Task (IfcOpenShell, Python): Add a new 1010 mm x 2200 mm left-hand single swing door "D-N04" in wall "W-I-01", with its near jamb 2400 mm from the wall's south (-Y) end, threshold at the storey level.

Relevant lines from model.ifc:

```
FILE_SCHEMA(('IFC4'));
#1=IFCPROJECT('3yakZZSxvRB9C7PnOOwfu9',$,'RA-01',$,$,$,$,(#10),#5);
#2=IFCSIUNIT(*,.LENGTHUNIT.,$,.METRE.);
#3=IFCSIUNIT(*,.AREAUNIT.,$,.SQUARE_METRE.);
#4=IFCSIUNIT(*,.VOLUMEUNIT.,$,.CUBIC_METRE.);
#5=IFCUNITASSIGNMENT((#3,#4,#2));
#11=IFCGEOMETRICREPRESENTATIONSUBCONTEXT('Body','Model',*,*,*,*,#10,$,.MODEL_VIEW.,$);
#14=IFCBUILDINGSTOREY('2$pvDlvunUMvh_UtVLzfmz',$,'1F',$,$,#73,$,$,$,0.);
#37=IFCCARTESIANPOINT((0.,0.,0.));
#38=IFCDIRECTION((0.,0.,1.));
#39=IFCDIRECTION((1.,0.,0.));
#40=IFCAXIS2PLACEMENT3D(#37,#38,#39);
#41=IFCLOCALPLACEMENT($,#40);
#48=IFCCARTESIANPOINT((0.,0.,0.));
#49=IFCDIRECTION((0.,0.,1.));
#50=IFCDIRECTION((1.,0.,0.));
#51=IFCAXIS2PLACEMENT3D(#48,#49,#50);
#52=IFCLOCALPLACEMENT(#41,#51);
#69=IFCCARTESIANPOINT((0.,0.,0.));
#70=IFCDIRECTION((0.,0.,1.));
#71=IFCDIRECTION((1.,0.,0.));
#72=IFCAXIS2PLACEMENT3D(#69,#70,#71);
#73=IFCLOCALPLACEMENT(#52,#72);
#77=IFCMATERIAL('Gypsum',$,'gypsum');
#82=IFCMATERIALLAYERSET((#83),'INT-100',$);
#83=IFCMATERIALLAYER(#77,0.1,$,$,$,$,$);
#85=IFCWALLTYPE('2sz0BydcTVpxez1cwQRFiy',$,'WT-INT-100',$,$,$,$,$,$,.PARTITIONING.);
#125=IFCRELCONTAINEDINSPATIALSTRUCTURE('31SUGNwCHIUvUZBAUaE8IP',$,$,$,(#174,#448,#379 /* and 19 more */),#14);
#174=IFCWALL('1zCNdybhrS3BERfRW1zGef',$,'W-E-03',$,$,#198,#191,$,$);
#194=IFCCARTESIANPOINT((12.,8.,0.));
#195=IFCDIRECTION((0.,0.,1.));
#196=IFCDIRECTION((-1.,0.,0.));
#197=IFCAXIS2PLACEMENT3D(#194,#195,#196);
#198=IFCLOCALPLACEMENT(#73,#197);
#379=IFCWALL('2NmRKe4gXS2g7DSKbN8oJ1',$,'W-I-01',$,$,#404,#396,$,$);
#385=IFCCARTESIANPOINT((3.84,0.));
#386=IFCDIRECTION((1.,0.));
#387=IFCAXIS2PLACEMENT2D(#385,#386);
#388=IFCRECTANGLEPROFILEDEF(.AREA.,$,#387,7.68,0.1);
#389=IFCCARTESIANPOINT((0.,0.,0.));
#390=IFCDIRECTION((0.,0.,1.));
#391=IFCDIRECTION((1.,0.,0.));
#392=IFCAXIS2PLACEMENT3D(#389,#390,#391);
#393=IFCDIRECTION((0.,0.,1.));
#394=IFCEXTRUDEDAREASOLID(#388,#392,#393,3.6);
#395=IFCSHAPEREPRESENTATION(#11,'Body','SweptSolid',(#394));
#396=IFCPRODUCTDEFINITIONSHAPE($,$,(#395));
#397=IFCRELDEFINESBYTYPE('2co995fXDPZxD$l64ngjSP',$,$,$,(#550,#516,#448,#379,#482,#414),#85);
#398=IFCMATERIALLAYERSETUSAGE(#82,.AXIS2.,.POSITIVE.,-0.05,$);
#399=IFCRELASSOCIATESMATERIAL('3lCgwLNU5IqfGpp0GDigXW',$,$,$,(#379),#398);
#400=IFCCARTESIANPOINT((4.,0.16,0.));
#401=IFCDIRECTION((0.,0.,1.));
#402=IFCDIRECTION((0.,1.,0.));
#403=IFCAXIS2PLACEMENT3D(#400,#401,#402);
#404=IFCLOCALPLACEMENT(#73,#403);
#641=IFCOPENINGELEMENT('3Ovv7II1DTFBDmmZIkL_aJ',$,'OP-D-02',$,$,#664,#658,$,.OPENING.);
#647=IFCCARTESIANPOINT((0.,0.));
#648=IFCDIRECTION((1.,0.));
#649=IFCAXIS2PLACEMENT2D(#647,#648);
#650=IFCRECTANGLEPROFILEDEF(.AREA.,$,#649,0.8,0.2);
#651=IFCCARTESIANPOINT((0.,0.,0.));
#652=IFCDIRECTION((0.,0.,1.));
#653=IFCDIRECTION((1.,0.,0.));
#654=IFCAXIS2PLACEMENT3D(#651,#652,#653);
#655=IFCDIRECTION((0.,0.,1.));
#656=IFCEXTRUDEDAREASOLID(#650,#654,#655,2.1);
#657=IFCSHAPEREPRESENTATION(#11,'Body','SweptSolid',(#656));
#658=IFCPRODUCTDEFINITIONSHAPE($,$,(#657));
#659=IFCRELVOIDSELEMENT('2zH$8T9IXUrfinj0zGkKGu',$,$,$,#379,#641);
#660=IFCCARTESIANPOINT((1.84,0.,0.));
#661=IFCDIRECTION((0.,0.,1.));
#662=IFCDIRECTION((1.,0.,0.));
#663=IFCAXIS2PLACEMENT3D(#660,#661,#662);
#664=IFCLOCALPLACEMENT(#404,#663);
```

```python
import numpy as np
import ifcopenshell
import ifcopenshell.api.feature
import ifcopenshell.api.geometry
import ifcopenshell.api.root
import ifcopenshell.api.spatial
import ifcopenshell.geom
import ifcopenshell.util.element
import ifcopenshell.util.placement
import ifcopenshell.util.representation
import ifcopenshell.util.shape
import ifcopenshell.util.unit

model = ifcopenshell.open("model.ifc")
unit_scale = ifcopenshell.util.unit.calculate_unit_scale(model)
settings = ifcopenshell.geom.settings()


def volume(element):
    """Net volume in cubic metres, openings subtracted."""
    shape = ifcopenshell.geom.create_shape(settings, element)
    return ifcopenshell.util.shape.get_volume(shape.geometry)


wall = model.by_guid("2NmRKe4gXS2g7DSKbN8oJ1")
storey = ifcopenshell.util.element.get_container(wall, ifc_class="IfcBuildingStorey")
context = ifcopenshell.util.representation.get_context(model, "Model", "Body", "MODEL_VIEW")
before = volume(wall)

width, height, from_end, sill = 1.01, 2.2, 2.4, 0.0  # metres

# The wall runs along its own X axis, and the end named is its -X end.
wall_shape = ifcopenshell.geom.create_shape(settings, wall)
x, y, z = ifcopenshell.util.shape.get_vertices(wall_shape.geometry).T
start = x.min() + from_end
face, thickness = float(y.min()), float(y.max() - y.min())
wall_matrix = ifcopenshell.util.placement.get_local_placement(wall.ObjectPlacement)
level = ifcopenshell.util.placement.get_local_placement(storey.ObjectPlacement)[2, 3]


def in_wall(x, y):
    """Placement at x, y metres in the wall's axes, at sill height."""
    matrix = wall_matrix.copy()
    matrix[:, 3] = wall_matrix @ np.array([x / unit_scale, y / unit_scale, 0.0, 1.0])
    matrix[2, 3] = level + sill / unit_scale
    return matrix


# Opening: a box that overshoots both wall faces by 50 mm.
opening = ifcopenshell.api.root.create_entity(model, ifc_class="IfcOpeningElement", predefined_type="OPENING")
box = ifcopenshell.api.geometry.add_wall_representation(
    model, context=context, length=width, height=height, thickness=thickness + 0.1
)
ifcopenshell.api.geometry.assign_representation(model, product=opening, representation=box)
ifcopenshell.api.geometry.edit_object_placement(model, product=opening, matrix=in_wall(start, face - 0.05), is_si=False)
ifcopenshell.api.feature.add_feature(model, feature=opening, element=wall)

door = ifcopenshell.api.root.create_entity(model, ifc_class="IfcDoor", name="D-N04", predefined_type="DOOR")
door.OverallWidth, door.OverallHeight = width / unit_scale, height / unit_scale
door.OperationType = "SINGLE_SWING_LEFT"
body = ifcopenshell.api.geometry.add_door_representation(
    model,
    context=context,
    overall_width=door.OverallWidth,
    overall_height=door.OverallHeight,
    operation_type="SINGLE_SWING_LEFT",
    lining_properties={"LiningDepth": thickness / unit_scale, "ThresholdDepth": thickness / unit_scale},
)
ifcopenshell.api.geometry.assign_representation(model, product=door, representation=body)
ifcopenshell.api.spatial.assign_container(model, products=[door], relating_structure=storey)
ifcopenshell.api.feature.add_filling(model, opening=opening, element=door)

# The lining spans the wall, so the door starts at the wall face.
ifcopenshell.api.geometry.edit_object_placement(model, product=door, matrix=in_wall(start, face), is_si=False)

after = volume(wall)

print(f"wall volume {before:.3f} -> {after:.3f} m3")

model.write("model_rev.ifc")
```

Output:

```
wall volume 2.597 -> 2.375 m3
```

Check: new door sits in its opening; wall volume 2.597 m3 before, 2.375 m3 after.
